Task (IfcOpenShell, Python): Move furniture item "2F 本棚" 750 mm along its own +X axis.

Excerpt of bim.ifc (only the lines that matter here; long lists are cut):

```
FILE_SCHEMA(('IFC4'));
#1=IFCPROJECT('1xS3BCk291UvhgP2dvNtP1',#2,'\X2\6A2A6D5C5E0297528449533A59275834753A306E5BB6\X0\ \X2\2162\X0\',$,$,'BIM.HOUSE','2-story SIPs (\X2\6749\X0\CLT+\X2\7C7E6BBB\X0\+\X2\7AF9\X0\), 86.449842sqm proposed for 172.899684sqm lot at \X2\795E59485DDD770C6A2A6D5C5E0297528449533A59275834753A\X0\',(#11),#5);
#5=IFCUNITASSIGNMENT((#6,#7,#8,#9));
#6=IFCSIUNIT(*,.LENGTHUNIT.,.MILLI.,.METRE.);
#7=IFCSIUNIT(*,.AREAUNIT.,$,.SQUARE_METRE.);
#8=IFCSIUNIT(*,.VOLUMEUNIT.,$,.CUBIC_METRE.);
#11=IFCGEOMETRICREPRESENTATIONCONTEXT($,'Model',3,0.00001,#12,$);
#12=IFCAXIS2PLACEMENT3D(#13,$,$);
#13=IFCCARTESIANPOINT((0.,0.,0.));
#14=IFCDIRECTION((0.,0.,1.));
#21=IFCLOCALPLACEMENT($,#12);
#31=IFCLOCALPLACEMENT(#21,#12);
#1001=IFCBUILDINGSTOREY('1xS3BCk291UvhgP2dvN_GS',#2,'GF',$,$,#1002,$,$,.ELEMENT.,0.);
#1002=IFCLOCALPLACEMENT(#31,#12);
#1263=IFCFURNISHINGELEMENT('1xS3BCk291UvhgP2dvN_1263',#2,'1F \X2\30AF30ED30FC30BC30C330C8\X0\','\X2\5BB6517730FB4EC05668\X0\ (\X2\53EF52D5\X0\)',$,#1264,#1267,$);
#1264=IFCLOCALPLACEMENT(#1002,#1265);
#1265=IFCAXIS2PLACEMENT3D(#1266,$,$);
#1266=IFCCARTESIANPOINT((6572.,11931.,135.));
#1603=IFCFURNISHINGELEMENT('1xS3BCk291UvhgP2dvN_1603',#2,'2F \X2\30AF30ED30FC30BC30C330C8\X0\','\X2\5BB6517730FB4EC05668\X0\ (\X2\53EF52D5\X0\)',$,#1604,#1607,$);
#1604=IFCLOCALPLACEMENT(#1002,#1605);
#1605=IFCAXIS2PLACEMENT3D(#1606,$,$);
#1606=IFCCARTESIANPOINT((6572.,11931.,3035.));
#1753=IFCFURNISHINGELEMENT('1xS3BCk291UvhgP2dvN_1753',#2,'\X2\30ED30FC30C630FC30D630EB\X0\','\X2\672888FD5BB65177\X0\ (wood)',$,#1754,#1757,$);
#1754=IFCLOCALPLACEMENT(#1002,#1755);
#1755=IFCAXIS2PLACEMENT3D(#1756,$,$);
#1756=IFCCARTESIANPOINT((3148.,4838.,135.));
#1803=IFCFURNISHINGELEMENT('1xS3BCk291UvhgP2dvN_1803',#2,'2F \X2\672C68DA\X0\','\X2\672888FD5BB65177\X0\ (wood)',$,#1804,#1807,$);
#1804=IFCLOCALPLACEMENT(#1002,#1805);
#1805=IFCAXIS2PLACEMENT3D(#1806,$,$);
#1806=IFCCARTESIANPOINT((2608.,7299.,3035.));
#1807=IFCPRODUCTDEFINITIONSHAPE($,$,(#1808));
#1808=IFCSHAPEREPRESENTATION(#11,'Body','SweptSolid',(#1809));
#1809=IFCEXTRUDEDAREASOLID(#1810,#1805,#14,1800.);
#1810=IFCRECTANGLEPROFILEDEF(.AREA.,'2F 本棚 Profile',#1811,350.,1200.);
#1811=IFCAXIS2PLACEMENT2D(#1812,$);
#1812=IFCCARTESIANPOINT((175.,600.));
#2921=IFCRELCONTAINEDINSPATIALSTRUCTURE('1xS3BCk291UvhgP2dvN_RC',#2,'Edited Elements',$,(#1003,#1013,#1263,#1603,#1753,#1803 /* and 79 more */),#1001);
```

```python
import ifcopenshell
import ifcopenshell.api.geometry
import ifcopenshell.util.placement
import ifcopenshell.util.unit

model = ifcopenshell.open("bim.ifc")
unit_scale = ifcopenshell.util.unit.calculate_unit_scale(model)

item = model.by_guid("1xS3BCk291UvhgP2dvN_1803")
matrix = ifcopenshell.util.placement.get_local_placement(item.ObjectPlacement)
matrix[:3, 3] += matrix[:3, 0] * 0.75 / unit_scale
ifcopenshell.api.geometry.edit_object_placement(model, product=item, matrix=matrix, is_si=False)

print(ifcopenshell.util.placement.get_local_placement(item.ObjectPlacement).round(3) + 0.0)

model.write("bim_updated.ifc")
```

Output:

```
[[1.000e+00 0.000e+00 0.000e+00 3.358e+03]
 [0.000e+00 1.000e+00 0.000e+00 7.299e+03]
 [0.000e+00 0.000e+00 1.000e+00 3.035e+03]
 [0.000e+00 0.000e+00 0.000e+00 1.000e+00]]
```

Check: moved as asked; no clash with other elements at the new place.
